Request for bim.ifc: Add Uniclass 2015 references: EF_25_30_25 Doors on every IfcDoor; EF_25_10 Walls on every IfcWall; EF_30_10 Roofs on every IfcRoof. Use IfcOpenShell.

First a look at what the model holds.

```python
import ifcopenshell

model = ifcopenshell.open("bim.ifc")
print(model.schema)
print("classifications:", [c.Name for c in model.by_type("IfcClassification")])
for ifc_class in ("IfcDoor", "IfcRoof", "IfcStair", "IfcWall", "IfcWindow"):
    print(ifc_class, len(model.by_type(ifc_class)))
```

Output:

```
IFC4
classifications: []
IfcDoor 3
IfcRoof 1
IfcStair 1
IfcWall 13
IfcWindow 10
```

```python
import ifcopenshell
import ifcopenshell.api.classification

model = ifcopenshell.open("bim.ifc")

system = ifcopenshell.api.classification.add_classification(model, classification="Uniclass 2015")

codes = {
    "IfcDoor": ("EF_25_30_25", "Doors"),
    "IfcWall": ("EF_25_10", "Walls"),
    "IfcRoof": ("EF_30_10", "Roofs"),
}
for ifc_class, (code, name) in codes.items():
    products = model.by_type(ifc_class)
    ifcopenshell.api.classification.add_reference(
        model, products=products, classification=system, identification=code, name=name
    )
    print(code, len(products))

model.write("bim_v2.ifc")
```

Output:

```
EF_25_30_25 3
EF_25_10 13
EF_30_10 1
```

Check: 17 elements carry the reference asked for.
